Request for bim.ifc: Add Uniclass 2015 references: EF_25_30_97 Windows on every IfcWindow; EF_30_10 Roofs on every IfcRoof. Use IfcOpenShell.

First a look at what the model holds.

```python
import ifcopenshell

model = ifcopenshell.open("bim.ifc")
print(model.schema)
print("classifications:", [c.Name for c in model.by_type("IfcClassification")])
for ifc_class in ("IfcDoor", "IfcRoof", "IfcStair", "IfcWall", "IfcWindow"):
    print(ifc_class, len(model.by_type(ifc_class)))
```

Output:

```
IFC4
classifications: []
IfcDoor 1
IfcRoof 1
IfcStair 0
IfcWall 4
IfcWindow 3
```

```python
import ifcopenshell
import ifcopenshell.api.classification

model = ifcopenshell.open("bim.ifc")

system = ifcopenshell.api.classification.add_classification(model, classification="Uniclass 2015")

codes = {
    "IfcWindow": ("EF_25_30_97", "Windows"),
    "IfcRoof": ("EF_30_10", "Roofs"),
}
for ifc_class, (code, name) in codes.items():
    products = model.by_type(ifc_class)
    ifcopenshell.api.classification.add_reference(
        model, products=products, classification=system, identification=code, name=name
    )
    print(code, len(products))

model.write("bim_rev.ifc")
```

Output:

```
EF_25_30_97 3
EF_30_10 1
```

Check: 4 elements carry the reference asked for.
